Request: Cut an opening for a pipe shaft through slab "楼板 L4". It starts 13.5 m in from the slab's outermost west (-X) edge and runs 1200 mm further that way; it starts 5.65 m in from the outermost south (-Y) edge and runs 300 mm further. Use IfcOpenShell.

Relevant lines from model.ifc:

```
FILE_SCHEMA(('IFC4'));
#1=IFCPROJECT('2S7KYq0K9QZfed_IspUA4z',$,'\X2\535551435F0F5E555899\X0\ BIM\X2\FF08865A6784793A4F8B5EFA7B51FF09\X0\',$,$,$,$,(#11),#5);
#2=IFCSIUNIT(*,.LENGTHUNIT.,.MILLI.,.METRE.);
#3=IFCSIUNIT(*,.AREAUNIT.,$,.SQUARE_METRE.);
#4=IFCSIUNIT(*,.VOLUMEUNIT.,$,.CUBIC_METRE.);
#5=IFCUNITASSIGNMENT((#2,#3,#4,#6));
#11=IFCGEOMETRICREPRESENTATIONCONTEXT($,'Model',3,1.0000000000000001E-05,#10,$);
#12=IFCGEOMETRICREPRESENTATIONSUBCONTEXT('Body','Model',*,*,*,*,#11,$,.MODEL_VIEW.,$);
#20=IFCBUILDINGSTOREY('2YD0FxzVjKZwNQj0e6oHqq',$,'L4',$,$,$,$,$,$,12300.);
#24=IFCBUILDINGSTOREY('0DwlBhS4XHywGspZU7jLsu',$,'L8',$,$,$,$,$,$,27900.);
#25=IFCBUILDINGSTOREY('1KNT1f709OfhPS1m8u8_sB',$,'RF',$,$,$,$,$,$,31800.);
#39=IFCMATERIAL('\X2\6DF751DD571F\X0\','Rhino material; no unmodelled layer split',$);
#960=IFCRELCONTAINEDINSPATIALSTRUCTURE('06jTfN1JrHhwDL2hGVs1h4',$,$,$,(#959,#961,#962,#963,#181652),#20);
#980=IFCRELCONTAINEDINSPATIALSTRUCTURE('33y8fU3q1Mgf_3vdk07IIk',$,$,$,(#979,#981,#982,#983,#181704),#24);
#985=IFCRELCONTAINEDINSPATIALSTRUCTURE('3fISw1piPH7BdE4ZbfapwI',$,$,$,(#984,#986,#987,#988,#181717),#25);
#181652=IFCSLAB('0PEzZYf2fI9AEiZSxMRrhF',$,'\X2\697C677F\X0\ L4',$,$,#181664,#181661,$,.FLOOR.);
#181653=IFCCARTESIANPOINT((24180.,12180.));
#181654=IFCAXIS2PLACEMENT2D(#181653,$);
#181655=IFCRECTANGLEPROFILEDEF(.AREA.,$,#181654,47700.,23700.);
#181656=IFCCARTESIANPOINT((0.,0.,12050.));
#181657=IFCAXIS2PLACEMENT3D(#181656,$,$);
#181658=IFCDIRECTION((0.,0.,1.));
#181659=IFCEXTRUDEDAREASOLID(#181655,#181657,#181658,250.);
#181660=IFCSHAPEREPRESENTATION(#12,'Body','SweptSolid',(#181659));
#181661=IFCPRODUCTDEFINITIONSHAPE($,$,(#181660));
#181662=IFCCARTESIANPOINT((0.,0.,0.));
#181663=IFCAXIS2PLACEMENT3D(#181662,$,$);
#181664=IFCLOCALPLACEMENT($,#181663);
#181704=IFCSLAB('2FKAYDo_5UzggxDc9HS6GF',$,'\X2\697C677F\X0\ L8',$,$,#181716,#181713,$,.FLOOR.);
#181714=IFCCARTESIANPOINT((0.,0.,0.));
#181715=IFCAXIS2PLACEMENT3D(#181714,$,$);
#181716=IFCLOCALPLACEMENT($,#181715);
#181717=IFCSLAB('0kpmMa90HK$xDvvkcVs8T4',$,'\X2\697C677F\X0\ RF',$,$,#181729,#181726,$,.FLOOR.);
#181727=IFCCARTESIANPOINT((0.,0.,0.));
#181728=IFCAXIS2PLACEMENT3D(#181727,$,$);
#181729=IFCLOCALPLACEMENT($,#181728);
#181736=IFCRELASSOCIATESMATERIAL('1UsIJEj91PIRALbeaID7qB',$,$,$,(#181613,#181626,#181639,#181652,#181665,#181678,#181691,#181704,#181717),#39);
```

```python
import numpy as np
import ifcopenshell
import ifcopenshell.api.feature
import ifcopenshell.api.geometry
import ifcopenshell.api.root
import ifcopenshell.geom
import ifcopenshell.util.placement
import ifcopenshell.util.representation
import ifcopenshell.util.shape
import ifcopenshell.util.unit

model = ifcopenshell.open("model.ifc")
unit_scale = ifcopenshell.util.unit.calculate_unit_scale(model)
settings = ifcopenshell.geom.settings()


def volume(element):
    """Net volume in cubic metres, openings subtracted."""
    shape = ifcopenshell.geom.create_shape(settings, element)
    return ifcopenshell.util.shape.get_volume(shape.geometry)


slab = model.by_guid("0PEzZYf2fI9AEiZSxMRrhF")
before = volume(slab)

# Extent in the slab's own axes, in metres. The edges named are its -X and -Y sides.
slab_shape = ifcopenshell.geom.create_shape(settings, slab)
vertices = ifcopenshell.util.shape.get_vertices(slab_shape.geometry)
x_min, y_min, bottom = vertices.min(axis=0)
top = vertices[:, 2].max()

opening = ifcopenshell.api.root.create_entity(model, ifc_class="IfcOpeningElement", name="Pipe shaft opening", predefined_type="OPENING")
context = ifcopenshell.util.representation.get_context(model, "Model", "Body", "MODEL_VIEW")
width, depth = 1.2, 0.3
outline = [(0.0, 0.0), (width, 0.0), (width, depth), (0.0, depth), (0.0, 0.0)]
# Overshoot both faces by 50 mm so the cut is clean.
shape = ifcopenshell.api.geometry.add_slab_representation(
    model, context=context, depth=top - bottom + 0.1, polyline=outline
)
ifcopenshell.api.geometry.assign_representation(model, product=opening, representation=shape)

matrix = ifcopenshell.util.placement.get_local_placement(slab.ObjectPlacement)
matrix[:, 3] = matrix @ np.append(np.array([x_min + 13.5, y_min + 5.65, bottom - 0.05]) / unit_scale, 1.0)
ifcopenshell.api.geometry.edit_object_placement(model, product=opening, matrix=matrix, is_si=False)
ifcopenshell.api.feature.add_feature(model, feature=opening, element=slab)

after = volume(slab)

print(f"slab volume {before:.3f} -> {after:.3f} m3")

model.write("model-out.ifc")
```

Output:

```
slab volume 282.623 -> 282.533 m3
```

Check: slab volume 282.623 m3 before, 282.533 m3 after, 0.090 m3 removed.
